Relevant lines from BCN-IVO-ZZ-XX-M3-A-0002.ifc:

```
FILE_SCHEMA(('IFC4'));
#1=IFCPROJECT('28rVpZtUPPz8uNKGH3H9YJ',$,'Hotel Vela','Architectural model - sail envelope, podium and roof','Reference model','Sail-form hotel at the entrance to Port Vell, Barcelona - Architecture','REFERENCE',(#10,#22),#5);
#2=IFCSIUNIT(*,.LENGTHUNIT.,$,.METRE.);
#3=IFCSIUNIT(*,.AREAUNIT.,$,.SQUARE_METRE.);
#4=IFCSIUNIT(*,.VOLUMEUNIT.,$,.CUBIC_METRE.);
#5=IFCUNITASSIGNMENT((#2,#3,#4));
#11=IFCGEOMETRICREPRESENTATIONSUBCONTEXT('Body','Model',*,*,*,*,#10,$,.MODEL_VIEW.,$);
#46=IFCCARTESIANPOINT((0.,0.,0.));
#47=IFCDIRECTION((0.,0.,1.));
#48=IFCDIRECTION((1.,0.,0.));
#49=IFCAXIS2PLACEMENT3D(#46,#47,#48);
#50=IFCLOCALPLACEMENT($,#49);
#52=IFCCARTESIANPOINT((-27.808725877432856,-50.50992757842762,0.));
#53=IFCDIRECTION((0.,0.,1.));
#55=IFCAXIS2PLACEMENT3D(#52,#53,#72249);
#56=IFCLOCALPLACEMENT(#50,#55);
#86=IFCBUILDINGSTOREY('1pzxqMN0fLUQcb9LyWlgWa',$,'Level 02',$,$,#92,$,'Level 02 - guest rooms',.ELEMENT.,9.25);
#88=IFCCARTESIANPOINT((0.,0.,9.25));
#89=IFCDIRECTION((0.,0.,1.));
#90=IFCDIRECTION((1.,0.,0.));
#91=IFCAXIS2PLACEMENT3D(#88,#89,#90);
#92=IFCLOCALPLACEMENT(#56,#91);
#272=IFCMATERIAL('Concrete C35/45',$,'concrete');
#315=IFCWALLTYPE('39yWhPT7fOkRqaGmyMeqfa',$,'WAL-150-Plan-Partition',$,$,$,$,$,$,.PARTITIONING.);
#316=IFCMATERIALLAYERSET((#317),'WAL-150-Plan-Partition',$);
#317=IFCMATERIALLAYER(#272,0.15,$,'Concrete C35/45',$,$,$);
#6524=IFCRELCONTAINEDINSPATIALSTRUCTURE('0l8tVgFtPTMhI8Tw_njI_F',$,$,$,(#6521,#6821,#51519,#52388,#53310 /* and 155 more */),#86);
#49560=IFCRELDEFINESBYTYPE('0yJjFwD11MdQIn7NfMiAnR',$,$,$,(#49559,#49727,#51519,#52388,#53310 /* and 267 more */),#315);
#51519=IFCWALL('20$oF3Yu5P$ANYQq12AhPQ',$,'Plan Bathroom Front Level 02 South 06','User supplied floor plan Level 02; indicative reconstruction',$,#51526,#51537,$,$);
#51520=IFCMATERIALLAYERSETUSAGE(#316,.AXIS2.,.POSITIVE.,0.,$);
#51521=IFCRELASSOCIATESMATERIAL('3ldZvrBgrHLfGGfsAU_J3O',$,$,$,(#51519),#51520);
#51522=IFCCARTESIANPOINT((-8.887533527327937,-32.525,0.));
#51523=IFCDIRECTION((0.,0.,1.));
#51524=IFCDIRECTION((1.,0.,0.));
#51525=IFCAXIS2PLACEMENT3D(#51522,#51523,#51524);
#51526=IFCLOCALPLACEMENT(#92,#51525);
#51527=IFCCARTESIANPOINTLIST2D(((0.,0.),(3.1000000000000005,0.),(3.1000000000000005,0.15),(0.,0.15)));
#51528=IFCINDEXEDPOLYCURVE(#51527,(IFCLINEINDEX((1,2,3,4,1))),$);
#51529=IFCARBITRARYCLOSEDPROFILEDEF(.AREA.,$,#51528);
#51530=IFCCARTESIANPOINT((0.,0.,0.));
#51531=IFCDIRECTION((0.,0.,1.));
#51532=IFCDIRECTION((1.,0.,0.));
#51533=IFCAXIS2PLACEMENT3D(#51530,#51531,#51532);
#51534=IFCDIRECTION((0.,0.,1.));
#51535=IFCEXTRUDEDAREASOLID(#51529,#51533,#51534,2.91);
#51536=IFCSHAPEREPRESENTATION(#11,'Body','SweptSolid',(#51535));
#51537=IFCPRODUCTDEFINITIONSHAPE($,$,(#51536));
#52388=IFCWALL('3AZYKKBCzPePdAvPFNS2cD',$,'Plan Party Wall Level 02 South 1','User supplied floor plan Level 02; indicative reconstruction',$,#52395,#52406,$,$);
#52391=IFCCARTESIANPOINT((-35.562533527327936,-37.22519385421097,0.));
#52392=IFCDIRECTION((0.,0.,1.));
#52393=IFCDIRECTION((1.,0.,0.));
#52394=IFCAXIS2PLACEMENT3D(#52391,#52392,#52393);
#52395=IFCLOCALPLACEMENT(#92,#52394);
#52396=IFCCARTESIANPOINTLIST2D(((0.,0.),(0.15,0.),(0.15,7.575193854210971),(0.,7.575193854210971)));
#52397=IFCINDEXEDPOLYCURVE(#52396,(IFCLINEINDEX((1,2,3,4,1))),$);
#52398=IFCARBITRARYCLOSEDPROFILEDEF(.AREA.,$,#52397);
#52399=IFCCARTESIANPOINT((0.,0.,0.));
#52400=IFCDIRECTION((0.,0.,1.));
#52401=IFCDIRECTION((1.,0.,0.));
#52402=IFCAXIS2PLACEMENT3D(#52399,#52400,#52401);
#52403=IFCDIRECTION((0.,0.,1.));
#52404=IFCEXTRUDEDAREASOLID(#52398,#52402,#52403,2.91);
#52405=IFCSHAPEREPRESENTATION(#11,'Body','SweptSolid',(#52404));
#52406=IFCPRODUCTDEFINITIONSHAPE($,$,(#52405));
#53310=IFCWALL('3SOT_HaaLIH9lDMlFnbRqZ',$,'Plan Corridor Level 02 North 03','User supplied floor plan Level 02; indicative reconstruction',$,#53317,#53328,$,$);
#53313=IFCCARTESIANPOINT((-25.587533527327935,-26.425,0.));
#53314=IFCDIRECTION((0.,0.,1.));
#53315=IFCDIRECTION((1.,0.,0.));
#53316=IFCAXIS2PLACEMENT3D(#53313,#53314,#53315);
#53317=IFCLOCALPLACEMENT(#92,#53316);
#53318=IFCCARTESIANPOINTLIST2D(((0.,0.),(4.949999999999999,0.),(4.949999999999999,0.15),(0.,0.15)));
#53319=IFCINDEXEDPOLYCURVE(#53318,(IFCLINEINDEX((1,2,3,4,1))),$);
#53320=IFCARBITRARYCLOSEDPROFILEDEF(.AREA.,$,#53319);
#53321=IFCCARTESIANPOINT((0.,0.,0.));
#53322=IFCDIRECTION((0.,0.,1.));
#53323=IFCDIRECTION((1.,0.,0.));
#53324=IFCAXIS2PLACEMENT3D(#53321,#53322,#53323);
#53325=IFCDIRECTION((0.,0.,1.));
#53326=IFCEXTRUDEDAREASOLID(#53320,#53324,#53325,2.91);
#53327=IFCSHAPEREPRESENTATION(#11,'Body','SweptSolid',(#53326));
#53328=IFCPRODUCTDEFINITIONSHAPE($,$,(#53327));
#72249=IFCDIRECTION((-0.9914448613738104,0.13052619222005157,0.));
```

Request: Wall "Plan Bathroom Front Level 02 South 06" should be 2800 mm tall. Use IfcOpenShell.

```python
import ifcopenshell
import ifcopenshell.geom
import ifcopenshell.util.representation
import ifcopenshell.util.shape

model = ifcopenshell.open("BCN-IVO-ZZ-XX-M3-A-0002.ifc")
settings = ifcopenshell.geom.settings()


def volume(element):
    """Net volume in cubic metres, openings subtracted."""
    shape = ifcopenshell.geom.create_shape(settings, element)
    return ifcopenshell.util.shape.get_volume(shape.geometry)


wall = model.by_guid("20$oF3Yu5P$ANYQq12AhPQ")
before = volume(wall)

body = ifcopenshell.util.representation.get_representation(wall, "Model", "Body")
solid = body.Items[0]
old_height = solid.Depth
solid.Depth = 2.8
after = volume(wall)

print(f"height {old_height:g} -> {solid.Depth:g}, volume {before:.3f} -> {after:.3f} m3")

model.write("BCN-IVO-ZZ-XX-M3-A-0002_updated.ifc")
```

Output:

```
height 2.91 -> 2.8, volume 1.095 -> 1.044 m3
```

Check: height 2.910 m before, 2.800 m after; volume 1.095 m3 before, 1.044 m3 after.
